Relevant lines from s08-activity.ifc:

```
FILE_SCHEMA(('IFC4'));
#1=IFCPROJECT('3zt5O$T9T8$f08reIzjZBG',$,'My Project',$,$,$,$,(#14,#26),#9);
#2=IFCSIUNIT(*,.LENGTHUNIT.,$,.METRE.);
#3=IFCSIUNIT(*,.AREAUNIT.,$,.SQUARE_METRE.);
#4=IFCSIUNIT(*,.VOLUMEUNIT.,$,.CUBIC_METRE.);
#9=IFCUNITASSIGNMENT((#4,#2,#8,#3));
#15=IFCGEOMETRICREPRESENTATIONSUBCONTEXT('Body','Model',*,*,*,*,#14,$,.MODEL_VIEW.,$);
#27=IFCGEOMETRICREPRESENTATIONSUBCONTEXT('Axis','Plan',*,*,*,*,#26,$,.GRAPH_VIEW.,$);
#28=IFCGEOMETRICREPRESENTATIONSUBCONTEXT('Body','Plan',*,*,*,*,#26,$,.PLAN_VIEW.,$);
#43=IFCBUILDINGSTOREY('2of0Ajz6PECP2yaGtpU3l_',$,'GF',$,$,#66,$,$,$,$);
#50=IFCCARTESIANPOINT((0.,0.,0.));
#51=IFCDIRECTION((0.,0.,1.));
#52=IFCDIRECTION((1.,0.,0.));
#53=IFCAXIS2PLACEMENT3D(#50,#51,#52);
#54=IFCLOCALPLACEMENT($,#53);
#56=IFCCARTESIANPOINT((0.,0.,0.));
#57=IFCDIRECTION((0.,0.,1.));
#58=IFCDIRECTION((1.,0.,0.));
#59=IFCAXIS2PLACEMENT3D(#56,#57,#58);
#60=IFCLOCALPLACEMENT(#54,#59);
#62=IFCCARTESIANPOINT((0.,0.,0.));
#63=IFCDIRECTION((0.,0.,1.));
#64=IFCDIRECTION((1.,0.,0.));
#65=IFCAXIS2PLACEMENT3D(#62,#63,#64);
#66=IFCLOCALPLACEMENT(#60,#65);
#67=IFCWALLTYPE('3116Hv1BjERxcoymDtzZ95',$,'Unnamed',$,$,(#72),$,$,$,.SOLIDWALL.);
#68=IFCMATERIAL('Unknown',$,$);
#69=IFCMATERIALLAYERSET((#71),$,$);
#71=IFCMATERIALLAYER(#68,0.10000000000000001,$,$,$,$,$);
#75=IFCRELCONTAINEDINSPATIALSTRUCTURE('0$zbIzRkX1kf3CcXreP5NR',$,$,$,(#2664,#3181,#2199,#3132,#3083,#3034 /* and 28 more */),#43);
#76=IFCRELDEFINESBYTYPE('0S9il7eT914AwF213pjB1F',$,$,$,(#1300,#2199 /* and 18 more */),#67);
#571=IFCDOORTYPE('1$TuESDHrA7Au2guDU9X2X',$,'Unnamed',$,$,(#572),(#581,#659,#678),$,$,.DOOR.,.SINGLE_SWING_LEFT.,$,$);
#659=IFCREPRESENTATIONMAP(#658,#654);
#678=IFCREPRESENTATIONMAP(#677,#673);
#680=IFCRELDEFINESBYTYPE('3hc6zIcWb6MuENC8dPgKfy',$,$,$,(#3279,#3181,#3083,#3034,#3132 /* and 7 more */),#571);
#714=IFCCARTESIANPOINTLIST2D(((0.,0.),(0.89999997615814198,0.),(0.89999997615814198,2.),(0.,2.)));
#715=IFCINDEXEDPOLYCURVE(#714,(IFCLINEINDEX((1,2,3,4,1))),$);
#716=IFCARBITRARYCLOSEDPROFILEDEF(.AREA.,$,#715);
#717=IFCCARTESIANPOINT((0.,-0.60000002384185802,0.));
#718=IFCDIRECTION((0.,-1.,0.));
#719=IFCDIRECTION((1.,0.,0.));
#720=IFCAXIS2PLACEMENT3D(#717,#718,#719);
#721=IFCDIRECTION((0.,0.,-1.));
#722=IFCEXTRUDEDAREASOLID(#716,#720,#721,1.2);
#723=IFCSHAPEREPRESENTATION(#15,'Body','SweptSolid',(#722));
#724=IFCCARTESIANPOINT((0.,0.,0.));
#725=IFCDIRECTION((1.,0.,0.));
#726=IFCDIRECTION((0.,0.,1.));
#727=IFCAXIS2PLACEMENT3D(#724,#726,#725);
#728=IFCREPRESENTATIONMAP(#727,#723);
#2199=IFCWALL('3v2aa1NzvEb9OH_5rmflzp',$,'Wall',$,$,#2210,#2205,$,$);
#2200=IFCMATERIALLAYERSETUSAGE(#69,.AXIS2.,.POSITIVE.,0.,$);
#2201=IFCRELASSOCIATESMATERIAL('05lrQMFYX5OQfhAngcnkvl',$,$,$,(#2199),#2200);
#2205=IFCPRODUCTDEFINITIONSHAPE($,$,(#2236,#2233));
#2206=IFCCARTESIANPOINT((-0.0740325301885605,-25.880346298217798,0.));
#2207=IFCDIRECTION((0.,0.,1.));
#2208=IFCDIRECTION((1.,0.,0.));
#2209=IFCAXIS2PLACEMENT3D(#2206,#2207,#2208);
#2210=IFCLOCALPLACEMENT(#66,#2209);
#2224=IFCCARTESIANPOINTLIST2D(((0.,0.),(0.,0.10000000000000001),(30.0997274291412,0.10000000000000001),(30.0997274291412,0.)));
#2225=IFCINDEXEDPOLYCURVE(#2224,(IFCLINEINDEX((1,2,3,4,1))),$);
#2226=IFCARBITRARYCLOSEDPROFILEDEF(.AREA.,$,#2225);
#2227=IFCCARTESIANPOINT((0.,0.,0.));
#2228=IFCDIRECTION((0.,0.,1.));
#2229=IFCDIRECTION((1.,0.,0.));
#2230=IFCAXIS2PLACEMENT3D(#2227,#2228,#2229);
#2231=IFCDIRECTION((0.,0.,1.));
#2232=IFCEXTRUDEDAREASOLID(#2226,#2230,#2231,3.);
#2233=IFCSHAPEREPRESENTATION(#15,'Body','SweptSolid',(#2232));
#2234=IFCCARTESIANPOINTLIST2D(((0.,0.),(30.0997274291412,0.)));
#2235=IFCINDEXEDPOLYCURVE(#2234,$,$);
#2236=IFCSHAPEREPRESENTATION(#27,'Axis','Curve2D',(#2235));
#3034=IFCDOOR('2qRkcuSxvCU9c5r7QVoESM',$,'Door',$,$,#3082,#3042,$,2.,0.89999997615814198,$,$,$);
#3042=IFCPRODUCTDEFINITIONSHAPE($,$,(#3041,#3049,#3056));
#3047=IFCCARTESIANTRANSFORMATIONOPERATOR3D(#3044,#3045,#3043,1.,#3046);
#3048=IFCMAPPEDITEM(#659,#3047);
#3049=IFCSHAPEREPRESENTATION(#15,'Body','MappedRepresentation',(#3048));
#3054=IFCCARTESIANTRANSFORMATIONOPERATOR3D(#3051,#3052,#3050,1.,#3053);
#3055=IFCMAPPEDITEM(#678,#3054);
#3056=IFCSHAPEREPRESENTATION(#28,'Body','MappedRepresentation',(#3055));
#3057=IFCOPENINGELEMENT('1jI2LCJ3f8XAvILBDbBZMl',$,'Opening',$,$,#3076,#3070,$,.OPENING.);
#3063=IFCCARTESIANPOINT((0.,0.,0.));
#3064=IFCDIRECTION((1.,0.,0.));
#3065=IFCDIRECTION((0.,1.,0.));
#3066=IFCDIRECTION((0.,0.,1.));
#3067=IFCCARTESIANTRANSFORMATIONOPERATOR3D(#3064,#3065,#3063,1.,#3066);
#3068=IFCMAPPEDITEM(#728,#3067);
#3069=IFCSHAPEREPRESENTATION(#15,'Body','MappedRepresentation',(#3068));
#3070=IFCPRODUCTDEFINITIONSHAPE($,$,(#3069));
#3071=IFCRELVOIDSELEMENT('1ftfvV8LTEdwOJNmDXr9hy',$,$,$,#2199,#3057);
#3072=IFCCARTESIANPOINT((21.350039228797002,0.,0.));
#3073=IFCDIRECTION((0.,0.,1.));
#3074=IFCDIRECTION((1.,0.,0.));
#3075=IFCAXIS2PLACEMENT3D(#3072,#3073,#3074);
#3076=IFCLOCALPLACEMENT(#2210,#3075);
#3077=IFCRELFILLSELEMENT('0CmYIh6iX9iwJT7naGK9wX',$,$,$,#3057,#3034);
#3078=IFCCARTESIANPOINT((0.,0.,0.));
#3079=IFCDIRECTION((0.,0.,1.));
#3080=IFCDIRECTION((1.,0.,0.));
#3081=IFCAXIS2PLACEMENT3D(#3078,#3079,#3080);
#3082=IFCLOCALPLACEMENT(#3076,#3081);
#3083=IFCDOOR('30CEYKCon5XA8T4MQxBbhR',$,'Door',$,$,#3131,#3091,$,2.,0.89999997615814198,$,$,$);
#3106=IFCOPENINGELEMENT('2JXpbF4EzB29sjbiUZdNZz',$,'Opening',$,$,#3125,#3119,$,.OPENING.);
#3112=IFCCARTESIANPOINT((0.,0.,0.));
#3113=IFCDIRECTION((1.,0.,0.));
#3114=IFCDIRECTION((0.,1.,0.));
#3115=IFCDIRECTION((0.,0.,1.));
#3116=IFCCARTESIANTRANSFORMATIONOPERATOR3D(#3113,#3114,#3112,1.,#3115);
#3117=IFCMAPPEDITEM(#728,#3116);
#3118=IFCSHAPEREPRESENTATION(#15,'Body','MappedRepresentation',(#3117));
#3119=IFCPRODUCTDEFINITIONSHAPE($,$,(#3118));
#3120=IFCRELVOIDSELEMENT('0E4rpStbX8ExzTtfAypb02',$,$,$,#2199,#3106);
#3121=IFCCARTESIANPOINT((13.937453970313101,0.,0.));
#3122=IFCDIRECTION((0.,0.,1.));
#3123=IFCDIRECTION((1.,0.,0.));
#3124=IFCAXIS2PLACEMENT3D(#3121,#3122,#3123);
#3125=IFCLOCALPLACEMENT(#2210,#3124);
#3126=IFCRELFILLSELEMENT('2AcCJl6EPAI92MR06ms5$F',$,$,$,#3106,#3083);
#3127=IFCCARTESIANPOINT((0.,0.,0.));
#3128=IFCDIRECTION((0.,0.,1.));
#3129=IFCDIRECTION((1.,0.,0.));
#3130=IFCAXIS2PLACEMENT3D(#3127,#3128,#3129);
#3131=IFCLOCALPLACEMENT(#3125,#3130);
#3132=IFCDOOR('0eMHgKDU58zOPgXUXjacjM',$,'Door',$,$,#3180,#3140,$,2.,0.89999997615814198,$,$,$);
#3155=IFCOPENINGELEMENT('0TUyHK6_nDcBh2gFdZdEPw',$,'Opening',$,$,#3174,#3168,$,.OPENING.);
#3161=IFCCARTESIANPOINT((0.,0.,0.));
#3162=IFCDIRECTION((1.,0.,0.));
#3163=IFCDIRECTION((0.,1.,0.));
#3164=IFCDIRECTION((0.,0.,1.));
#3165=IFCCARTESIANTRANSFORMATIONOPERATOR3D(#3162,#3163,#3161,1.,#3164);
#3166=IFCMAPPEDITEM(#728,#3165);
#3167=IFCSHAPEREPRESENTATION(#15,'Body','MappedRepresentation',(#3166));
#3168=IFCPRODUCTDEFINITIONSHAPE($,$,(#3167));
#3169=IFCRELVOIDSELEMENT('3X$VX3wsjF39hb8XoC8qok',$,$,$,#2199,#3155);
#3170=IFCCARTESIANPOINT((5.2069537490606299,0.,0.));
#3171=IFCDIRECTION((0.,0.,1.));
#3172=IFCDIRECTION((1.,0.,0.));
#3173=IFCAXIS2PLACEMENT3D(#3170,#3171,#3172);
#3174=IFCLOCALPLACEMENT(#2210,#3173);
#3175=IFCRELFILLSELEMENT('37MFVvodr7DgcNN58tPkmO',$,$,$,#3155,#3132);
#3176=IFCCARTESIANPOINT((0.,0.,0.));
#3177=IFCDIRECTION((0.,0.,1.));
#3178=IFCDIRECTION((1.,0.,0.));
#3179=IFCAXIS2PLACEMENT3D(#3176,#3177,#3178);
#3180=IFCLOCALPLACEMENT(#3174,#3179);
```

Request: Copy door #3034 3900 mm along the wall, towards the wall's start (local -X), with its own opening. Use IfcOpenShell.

```python
import ifcopenshell
import ifcopenshell.api.feature
import ifcopenshell.api.geometry
import ifcopenshell.api.root
import ifcopenshell.geom
import ifcopenshell.util.element
import ifcopenshell.util.placement
import ifcopenshell.util.shape

model = ifcopenshell.open("s08-activity.ifc")
settings = ifcopenshell.geom.settings()


def volume(element):
    """Net volume in cubic metres, openings subtracted."""
    shape = ifcopenshell.geom.create_shape(settings, element)
    return ifcopenshell.util.shape.get_volume(shape.geometry)


door = model.by_guid("2qRkcuSxvCU9c5r7QVoESM")
opening = door.FillsVoids[0].RelatingOpeningElement
wall = opening.VoidsElements[0].RelatingBuildingElement
before = volume(wall)
shift = ifcopenshell.util.placement.get_local_placement(wall.ObjectPlacement)[:3, 0] * -3.9

# copy_class copies the void relationship, type, container and properties, but no geometry.
new_opening = ifcopenshell.api.root.copy_class(model, product=opening)
new_opening.Representation = ifcopenshell.util.element.copy_deep(
    model, opening.Representation, exclude=["IfcGeometricRepresentationContext", "IfcRepresentationMap"]
)
new_door = ifcopenshell.api.root.copy_class(model, product=door)
new_door.Representation = ifcopenshell.util.element.copy_deep(
    model, door.Representation, exclude=["IfcGeometricRepresentationContext", "IfcRepresentationMap"]
)
ifcopenshell.api.feature.add_filling(model, opening=new_opening, element=new_door)

for old, new in ((opening, new_opening), (door, new_door)):
    matrix = ifcopenshell.util.placement.get_local_placement(old.ObjectPlacement)
    matrix[:3, 3] += shift
    ifcopenshell.api.geometry.edit_object_placement(model, product=new, matrix=matrix, is_si=False)

after = volume(wall)

print(f"wall volume {before:.3f} -> {after:.3f} m3")

model.write("s08-activity_v2.ifc")
```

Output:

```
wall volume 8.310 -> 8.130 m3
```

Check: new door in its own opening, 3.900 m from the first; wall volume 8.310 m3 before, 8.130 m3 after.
